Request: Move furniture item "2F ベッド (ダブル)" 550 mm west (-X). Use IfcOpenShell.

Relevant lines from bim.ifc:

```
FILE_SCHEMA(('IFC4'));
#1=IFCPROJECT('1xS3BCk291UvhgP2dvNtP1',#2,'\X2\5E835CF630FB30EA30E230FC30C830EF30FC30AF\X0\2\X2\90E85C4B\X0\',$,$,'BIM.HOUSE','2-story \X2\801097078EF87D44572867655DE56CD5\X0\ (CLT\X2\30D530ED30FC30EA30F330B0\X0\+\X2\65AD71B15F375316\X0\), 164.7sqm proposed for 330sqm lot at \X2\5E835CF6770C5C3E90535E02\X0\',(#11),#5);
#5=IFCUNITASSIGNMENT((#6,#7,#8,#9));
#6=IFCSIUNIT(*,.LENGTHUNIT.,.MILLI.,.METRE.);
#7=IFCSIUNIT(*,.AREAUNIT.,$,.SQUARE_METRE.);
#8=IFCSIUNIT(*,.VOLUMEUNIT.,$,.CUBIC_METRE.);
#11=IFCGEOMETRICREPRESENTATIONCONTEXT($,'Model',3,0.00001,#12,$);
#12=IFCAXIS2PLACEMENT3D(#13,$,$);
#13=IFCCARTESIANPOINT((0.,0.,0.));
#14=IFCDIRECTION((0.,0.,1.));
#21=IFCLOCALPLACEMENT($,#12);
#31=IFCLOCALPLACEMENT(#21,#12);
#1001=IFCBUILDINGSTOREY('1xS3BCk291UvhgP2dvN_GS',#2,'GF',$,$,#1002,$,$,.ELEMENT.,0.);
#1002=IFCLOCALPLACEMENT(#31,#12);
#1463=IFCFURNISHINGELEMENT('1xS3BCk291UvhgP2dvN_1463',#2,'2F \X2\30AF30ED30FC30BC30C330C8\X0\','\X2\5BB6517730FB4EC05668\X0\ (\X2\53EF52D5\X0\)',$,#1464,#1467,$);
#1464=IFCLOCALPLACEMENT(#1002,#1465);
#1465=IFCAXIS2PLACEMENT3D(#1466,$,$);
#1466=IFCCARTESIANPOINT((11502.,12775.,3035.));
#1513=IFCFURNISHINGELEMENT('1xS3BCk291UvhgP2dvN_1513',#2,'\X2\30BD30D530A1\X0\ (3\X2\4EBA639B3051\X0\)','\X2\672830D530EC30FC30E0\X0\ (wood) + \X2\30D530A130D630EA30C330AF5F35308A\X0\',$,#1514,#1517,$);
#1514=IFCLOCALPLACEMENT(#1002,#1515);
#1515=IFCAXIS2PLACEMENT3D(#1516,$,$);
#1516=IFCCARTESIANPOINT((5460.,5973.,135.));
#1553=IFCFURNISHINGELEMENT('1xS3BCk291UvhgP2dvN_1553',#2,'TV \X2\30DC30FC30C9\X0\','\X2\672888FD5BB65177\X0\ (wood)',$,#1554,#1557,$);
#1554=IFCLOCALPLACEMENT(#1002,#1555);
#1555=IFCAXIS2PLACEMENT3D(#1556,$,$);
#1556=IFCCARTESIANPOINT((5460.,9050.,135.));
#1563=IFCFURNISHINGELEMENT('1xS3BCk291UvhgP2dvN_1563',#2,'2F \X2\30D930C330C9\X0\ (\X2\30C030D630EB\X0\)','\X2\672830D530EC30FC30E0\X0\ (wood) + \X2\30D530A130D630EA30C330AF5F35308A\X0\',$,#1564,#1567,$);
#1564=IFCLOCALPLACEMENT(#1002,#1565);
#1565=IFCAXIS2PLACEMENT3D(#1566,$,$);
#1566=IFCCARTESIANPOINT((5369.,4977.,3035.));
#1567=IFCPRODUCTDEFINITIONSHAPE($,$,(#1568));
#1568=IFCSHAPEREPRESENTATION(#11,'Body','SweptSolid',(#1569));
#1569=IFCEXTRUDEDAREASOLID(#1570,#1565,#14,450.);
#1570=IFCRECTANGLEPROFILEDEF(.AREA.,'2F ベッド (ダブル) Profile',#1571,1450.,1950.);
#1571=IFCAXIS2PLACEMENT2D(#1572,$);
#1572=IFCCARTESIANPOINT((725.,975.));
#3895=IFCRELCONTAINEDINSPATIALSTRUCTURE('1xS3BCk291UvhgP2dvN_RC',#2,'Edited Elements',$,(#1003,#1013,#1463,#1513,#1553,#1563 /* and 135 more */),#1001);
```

```python
import ifcopenshell
import ifcopenshell.api.geometry
import ifcopenshell.util.placement
import ifcopenshell.util.unit

model = ifcopenshell.open("bim.ifc")
unit_scale = ifcopenshell.util.unit.calculate_unit_scale(model)

item = model.by_guid("1xS3BCk291UvhgP2dvN_1563")
matrix = ifcopenshell.util.placement.get_local_placement(item.ObjectPlacement)
matrix[0, 3] -= 0.55 / unit_scale
ifcopenshell.api.geometry.edit_object_placement(model, product=item, matrix=matrix, is_si=False)

print(ifcopenshell.util.placement.get_local_placement(item.ObjectPlacement).round(3) + 0.0)

model.write("bim_v2.ifc")
```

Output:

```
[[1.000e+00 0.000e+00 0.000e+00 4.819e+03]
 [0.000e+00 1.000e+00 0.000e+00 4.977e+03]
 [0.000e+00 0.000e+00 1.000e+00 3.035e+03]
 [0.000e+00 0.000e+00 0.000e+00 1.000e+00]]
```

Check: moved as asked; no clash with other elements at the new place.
